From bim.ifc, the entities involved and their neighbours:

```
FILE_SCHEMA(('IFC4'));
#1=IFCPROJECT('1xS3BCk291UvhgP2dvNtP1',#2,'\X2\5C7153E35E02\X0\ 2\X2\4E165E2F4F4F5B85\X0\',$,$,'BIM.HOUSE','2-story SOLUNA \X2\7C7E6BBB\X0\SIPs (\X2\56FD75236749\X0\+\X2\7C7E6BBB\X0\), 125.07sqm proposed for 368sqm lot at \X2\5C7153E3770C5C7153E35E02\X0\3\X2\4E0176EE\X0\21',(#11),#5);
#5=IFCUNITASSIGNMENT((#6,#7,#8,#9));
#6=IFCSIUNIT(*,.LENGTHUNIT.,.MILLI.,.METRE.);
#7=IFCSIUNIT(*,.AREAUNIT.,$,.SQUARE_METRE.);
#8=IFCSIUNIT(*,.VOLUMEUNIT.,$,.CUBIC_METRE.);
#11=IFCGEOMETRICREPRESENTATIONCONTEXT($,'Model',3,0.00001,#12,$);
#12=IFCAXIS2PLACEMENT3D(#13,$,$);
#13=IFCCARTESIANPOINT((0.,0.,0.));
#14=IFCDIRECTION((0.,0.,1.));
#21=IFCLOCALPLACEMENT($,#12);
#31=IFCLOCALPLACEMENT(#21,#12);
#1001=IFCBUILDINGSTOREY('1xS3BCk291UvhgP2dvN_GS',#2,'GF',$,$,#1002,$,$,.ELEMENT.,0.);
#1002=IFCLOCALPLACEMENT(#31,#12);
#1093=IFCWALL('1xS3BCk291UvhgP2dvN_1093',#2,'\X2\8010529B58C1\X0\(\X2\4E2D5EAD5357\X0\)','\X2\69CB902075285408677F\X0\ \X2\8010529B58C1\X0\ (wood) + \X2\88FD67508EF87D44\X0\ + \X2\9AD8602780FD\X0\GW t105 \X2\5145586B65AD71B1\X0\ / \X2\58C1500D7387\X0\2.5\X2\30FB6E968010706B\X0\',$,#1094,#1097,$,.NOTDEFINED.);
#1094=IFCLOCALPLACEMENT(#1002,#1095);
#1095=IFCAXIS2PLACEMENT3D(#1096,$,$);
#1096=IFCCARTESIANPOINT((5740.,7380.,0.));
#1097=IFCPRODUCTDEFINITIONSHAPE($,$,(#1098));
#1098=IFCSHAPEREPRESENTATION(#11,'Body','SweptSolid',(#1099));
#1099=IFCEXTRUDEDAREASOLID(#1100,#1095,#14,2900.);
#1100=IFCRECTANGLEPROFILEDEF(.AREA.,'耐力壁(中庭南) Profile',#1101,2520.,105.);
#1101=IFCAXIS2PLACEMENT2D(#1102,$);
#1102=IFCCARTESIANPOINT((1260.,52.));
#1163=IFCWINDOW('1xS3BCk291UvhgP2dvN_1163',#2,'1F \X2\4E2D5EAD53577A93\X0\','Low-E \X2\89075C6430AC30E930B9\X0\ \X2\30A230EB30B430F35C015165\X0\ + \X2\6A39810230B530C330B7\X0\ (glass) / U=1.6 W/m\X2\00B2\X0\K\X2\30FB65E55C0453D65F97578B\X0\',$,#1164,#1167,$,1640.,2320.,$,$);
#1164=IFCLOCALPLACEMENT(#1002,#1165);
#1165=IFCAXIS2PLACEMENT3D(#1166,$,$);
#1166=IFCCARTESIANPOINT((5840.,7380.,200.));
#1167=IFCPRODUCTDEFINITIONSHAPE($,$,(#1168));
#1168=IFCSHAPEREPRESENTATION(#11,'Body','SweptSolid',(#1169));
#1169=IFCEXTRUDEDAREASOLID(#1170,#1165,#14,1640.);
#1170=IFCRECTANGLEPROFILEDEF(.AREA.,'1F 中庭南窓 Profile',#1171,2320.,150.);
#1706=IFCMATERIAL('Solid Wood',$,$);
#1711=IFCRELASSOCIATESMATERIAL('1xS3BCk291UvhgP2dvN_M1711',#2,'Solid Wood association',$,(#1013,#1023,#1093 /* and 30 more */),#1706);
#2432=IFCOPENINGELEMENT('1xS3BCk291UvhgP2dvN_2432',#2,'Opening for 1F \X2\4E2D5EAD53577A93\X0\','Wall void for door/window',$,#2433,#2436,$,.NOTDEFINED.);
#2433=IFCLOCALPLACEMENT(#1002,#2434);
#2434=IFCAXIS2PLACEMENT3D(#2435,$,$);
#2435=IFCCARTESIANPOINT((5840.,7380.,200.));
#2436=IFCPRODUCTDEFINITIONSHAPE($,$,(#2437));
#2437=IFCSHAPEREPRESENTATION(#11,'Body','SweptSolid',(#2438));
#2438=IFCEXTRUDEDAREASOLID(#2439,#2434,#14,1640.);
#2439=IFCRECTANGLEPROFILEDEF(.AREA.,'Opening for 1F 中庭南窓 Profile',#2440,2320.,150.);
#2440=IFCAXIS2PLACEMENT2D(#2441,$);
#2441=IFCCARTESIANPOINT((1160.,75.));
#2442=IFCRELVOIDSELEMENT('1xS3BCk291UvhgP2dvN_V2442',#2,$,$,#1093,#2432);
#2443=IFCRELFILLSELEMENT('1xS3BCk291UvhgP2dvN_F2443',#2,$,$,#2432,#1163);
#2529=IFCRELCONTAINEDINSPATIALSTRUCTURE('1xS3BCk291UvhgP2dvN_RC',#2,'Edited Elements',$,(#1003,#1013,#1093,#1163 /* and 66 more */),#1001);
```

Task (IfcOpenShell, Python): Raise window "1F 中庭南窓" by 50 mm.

```python
import numpy as np
import ifcopenshell
import ifcopenshell.api.geometry
import ifcopenshell.util.placement
import ifcopenshell.util.unit

model = ifcopenshell.open("bim.ifc")
unit_scale = ifcopenshell.util.unit.calculate_unit_scale(model)

window = model.by_guid("1xS3BCk291UvhgP2dvN_1163")
opening = window.FillsVoids[0].RelatingOpeningElement
dz = 0.05 / unit_scale

shift = np.array([0.0, 0.0, dz])
# The window is not placed relative to its opening, so move both.
for product in (opening, window):
    matrix = ifcopenshell.util.placement.get_local_placement(product.ObjectPlacement)
    matrix[:3, 3] += shift
    ifcopenshell.api.geometry.edit_object_placement(model, product=product, matrix=matrix, is_si=False)

print(f"moved by {dz * unit_scale:+.3f} m")

model.write("bim_updated.ifc")
```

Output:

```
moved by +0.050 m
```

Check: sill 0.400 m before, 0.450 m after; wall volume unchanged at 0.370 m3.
